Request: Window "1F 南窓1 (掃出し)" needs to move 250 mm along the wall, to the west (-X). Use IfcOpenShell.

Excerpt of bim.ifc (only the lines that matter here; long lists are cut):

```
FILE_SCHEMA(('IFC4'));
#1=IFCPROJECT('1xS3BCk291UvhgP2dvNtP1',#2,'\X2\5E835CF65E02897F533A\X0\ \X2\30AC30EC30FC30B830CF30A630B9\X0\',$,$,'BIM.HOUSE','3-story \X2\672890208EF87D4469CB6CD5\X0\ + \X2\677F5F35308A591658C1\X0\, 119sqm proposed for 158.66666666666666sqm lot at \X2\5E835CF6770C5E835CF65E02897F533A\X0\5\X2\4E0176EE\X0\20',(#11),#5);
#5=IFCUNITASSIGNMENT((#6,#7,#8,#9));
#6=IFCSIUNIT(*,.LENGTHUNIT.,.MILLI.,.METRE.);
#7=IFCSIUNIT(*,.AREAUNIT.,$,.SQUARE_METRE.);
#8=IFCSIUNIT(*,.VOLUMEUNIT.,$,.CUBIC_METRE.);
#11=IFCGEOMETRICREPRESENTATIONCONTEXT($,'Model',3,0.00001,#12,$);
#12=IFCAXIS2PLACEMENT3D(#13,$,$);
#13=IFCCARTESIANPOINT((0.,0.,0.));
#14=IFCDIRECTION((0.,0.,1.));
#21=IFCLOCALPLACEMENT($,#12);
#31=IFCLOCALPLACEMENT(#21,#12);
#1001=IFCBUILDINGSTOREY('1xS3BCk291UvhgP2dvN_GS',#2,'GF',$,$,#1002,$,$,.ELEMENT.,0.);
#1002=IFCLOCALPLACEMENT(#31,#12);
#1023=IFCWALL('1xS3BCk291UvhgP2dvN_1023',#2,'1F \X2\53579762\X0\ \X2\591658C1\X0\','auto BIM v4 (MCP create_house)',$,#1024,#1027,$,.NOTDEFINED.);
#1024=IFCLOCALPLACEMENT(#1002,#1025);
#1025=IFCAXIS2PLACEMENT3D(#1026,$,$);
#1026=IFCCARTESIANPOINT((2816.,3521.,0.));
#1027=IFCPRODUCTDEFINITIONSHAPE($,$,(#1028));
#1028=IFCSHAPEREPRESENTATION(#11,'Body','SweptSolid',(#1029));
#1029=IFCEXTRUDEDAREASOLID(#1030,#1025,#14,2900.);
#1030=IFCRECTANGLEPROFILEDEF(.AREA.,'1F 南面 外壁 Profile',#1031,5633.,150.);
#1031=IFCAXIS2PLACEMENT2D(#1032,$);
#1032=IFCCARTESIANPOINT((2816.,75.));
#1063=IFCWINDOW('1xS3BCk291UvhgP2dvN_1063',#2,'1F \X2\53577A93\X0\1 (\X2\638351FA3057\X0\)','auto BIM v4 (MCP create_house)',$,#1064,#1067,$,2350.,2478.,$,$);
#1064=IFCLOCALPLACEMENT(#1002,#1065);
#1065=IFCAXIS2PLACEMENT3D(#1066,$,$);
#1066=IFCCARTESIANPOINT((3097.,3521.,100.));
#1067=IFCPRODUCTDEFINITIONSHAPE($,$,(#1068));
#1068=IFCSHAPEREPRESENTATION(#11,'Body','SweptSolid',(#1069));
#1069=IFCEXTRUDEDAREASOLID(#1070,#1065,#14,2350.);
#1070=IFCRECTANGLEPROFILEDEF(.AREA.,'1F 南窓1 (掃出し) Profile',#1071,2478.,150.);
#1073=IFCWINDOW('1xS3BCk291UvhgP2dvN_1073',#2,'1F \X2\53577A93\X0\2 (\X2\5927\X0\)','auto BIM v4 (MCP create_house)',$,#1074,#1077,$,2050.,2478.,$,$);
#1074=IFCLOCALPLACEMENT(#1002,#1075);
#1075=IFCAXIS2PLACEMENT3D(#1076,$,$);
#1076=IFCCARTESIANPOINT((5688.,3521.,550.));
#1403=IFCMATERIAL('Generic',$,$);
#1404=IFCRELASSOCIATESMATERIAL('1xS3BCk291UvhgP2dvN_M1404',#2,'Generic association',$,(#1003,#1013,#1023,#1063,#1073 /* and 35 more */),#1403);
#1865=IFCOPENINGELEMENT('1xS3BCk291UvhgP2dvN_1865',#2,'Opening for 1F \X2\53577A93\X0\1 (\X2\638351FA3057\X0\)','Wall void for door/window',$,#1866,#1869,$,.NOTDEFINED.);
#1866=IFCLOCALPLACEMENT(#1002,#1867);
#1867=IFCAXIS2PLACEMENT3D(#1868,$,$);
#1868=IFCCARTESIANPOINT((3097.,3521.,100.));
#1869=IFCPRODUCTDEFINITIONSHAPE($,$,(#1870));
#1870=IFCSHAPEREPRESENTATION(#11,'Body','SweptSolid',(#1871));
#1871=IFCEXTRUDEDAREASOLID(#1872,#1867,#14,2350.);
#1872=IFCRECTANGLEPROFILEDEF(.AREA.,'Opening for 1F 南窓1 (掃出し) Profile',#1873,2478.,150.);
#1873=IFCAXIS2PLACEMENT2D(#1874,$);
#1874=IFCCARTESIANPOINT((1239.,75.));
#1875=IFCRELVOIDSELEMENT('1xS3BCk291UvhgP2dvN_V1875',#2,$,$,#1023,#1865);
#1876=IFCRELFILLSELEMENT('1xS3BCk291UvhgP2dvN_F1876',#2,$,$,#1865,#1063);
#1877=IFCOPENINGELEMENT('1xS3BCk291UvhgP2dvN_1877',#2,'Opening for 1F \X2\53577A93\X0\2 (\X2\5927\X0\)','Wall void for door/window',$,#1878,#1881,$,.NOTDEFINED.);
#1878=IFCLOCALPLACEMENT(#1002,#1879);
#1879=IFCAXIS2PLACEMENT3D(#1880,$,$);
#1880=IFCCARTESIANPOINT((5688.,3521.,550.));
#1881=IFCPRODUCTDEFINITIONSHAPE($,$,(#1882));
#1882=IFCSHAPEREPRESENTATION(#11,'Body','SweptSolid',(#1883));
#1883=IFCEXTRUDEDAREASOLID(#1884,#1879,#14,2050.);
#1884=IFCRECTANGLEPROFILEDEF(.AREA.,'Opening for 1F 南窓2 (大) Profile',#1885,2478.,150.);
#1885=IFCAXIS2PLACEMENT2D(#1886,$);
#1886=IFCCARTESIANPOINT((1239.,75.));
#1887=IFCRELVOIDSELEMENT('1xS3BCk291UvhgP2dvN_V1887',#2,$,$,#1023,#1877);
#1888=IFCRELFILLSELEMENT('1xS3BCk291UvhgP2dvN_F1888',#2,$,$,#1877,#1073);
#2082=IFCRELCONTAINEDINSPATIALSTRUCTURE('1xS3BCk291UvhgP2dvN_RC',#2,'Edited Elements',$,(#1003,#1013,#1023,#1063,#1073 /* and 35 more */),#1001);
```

```python
import ifcopenshell
import ifcopenshell.api.geometry
import ifcopenshell.util.placement

model = ifcopenshell.open("bim.ifc")

window = model.by_guid("1xS3BCk291UvhgP2dvN_1063")
opening = window.FillsVoids[0].RelatingOpeningElement
wall = opening.VoidsElements[0].RelatingBuildingElement

wall_matrix = ifcopenshell.util.placement.get_local_placement(wall.ObjectPlacement)
shift = wall_matrix[:3, 0] * -250.0
before = ifcopenshell.util.placement.get_local_placement(window.ObjectPlacement)[:3, 3].copy()

# The window is not placed relative to its opening, so move both.
for product in (opening, window):
    matrix = ifcopenshell.util.placement.get_local_placement(product.ObjectPlacement)
    matrix[:3, 3] += shift
    ifcopenshell.api.geometry.edit_object_placement(model, product=product, matrix=matrix, is_si=False)

after = ifcopenshell.util.placement.get_local_placement(window.ObjectPlacement)[:3, 3]
print("window moved by", (after - before).round(3) + 0.0)

model.write("bim_v2.ifc")
```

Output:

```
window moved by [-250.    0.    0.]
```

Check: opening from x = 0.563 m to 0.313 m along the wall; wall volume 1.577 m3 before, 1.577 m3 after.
